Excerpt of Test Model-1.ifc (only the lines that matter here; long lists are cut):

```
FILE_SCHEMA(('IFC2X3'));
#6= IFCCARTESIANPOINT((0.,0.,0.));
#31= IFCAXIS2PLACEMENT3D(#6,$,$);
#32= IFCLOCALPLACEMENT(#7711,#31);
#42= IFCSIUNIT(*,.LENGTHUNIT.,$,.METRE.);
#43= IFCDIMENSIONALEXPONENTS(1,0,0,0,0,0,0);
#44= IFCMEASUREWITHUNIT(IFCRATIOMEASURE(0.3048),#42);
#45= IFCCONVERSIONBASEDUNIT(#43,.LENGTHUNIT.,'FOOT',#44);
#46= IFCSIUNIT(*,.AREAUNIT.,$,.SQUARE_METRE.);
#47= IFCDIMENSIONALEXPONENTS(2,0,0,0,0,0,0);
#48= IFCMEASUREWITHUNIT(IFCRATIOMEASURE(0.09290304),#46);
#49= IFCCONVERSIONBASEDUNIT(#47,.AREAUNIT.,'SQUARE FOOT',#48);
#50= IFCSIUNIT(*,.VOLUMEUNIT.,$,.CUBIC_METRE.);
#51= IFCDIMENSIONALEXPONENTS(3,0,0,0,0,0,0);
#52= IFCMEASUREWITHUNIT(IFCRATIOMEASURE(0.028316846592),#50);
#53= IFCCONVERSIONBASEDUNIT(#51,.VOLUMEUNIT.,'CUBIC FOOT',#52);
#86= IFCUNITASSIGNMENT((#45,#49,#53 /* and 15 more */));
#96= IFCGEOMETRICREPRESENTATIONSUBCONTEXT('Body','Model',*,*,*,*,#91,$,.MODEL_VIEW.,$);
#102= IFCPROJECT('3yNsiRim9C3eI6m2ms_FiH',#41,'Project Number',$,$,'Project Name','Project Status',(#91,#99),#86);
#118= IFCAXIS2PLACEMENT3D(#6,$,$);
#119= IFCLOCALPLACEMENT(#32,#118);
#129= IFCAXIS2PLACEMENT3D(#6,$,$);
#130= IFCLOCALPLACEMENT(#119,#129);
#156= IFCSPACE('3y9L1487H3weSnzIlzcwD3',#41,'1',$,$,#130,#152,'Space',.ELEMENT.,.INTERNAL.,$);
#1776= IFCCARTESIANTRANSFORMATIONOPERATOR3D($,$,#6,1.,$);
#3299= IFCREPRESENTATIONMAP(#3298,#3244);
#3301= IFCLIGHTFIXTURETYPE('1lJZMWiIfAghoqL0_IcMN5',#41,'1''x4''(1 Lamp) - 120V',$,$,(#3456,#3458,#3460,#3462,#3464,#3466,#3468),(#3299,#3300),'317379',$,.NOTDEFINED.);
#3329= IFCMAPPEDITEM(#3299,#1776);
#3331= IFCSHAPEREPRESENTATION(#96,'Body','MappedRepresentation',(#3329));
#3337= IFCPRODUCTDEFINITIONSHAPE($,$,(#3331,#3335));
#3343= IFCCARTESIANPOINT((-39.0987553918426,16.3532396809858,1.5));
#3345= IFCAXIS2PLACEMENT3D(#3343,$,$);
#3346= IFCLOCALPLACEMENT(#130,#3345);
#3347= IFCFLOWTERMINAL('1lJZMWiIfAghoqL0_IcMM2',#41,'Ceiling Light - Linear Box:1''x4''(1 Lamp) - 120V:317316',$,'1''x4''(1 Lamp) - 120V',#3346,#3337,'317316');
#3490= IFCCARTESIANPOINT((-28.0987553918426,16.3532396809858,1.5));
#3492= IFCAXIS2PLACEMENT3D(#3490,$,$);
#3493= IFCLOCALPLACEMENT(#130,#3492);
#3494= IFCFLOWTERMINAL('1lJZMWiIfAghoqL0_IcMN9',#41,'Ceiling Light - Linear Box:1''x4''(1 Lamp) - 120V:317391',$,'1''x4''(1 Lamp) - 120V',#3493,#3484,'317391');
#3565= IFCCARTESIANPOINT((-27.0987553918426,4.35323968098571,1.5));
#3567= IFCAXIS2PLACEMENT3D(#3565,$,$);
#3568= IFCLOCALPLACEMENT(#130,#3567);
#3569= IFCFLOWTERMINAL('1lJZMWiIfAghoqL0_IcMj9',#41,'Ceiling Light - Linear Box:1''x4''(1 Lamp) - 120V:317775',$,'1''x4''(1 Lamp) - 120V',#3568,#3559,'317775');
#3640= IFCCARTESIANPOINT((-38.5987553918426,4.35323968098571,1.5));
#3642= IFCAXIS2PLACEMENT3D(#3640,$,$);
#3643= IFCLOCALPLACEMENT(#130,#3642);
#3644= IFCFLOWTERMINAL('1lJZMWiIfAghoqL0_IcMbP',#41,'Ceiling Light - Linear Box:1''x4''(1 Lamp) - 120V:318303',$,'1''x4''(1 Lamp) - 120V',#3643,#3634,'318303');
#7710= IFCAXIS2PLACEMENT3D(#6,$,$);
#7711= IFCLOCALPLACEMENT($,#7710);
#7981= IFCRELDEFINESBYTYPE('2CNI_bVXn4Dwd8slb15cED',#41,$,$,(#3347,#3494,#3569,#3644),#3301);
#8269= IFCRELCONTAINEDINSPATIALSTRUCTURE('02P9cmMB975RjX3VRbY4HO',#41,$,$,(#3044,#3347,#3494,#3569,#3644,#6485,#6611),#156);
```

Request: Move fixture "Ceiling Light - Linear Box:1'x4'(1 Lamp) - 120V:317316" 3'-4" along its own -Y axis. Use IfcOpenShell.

```python
import ifcopenshell
import ifcopenshell.api.geometry
import ifcopenshell.util.placement
import ifcopenshell.util.unit

model = ifcopenshell.open("Test Model-1.ifc")
unit_scale = ifcopenshell.util.unit.calculate_unit_scale(model)

item = model.by_guid("1lJZMWiIfAghoqL0_IcMM2")
matrix = ifcopenshell.util.placement.get_local_placement(item.ObjectPlacement)
matrix[:3, 3] -= matrix[:3, 1] * 40 * 0.0254 / unit_scale
ifcopenshell.api.geometry.edit_object_placement(model, product=item, matrix=matrix, is_si=False)

print(ifcopenshell.util.placement.get_local_placement(item.ObjectPlacement).round(3) + 0.0)

model.write("Test Model-1_edited.ifc")
```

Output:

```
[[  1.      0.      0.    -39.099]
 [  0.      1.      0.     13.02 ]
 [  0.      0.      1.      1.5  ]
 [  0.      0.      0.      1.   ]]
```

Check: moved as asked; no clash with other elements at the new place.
